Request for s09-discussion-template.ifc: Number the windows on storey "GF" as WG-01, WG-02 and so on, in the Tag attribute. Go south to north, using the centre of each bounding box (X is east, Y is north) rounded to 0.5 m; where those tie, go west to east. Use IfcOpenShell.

First a look at what the model holds.

```python
import ifcopenshell
import ifcopenshell.util.element
import ifcopenshell.util.placement

model = ifcopenshell.open("s09-discussion-template.ifc")
print(model.schema)
storey = next(s for s in model.by_type("IfcBuildingStorey") if s.Name == "GF")
windows = [e for e in ifcopenshell.util.element.get_decomposition(storey) if e.is_a("IfcWindow")]
for e in sorted(windows, key=lambda e: e.id()):
    origin = ifcopenshell.util.placement.get_local_placement(e.ObjectPlacement)[:3, 3]
    print(e.id(), e.Tag, e.Name, origin.round(2) + 0.0, sep=" | ")
```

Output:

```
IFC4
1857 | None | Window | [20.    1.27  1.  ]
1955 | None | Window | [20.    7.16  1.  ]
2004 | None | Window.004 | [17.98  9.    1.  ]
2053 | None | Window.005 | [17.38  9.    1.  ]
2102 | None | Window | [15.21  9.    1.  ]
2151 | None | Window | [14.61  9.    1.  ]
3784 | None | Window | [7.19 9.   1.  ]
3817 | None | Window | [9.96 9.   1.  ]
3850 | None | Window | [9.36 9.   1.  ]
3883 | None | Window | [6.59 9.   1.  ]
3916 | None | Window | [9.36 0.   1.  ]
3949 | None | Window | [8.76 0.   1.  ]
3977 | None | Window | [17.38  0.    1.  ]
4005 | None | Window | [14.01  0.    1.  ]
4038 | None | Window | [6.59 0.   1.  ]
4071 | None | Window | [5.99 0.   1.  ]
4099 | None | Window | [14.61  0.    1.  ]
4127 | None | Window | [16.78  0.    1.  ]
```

```python
import ifcopenshell
import ifcopenshell.geom
import ifcopenshell.util.element
import ifcopenshell.util.shape

model = ifcopenshell.open("s09-discussion-template.ifc")
settings = ifcopenshell.geom.settings()
settings.set("use-world-coords", True)


def centre(element):
    shape = ifcopenshell.geom.create_shape(settings, element)
    return ifcopenshell.util.shape.get_bbox_centroid(shape.geometry)


storey = next(s for s in model.by_type("IfcBuildingStorey") if s.Name == "GF")
windows = [e for e in ifcopenshell.util.element.get_decomposition(storey) if e.is_a("IfcWindow")]

# Insertion points can sit at a corner or the storey origin, so sort by the geometry (in metres).
centres = {e: centre(e) for e in windows}
windows.sort(key=lambda e: (round(centres[e][1] / 0.5), centres[e][0]))

for i, e in enumerate(windows, start=1):
    number = f"WG-{i:02d}"
    e.Tag = number
    print(e.id(), number)

model.write("s09-discussion-template-out.ifc")
```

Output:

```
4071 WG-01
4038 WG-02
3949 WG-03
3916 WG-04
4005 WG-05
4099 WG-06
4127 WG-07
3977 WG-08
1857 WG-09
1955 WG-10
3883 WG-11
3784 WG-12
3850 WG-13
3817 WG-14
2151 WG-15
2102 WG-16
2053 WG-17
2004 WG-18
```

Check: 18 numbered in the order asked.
